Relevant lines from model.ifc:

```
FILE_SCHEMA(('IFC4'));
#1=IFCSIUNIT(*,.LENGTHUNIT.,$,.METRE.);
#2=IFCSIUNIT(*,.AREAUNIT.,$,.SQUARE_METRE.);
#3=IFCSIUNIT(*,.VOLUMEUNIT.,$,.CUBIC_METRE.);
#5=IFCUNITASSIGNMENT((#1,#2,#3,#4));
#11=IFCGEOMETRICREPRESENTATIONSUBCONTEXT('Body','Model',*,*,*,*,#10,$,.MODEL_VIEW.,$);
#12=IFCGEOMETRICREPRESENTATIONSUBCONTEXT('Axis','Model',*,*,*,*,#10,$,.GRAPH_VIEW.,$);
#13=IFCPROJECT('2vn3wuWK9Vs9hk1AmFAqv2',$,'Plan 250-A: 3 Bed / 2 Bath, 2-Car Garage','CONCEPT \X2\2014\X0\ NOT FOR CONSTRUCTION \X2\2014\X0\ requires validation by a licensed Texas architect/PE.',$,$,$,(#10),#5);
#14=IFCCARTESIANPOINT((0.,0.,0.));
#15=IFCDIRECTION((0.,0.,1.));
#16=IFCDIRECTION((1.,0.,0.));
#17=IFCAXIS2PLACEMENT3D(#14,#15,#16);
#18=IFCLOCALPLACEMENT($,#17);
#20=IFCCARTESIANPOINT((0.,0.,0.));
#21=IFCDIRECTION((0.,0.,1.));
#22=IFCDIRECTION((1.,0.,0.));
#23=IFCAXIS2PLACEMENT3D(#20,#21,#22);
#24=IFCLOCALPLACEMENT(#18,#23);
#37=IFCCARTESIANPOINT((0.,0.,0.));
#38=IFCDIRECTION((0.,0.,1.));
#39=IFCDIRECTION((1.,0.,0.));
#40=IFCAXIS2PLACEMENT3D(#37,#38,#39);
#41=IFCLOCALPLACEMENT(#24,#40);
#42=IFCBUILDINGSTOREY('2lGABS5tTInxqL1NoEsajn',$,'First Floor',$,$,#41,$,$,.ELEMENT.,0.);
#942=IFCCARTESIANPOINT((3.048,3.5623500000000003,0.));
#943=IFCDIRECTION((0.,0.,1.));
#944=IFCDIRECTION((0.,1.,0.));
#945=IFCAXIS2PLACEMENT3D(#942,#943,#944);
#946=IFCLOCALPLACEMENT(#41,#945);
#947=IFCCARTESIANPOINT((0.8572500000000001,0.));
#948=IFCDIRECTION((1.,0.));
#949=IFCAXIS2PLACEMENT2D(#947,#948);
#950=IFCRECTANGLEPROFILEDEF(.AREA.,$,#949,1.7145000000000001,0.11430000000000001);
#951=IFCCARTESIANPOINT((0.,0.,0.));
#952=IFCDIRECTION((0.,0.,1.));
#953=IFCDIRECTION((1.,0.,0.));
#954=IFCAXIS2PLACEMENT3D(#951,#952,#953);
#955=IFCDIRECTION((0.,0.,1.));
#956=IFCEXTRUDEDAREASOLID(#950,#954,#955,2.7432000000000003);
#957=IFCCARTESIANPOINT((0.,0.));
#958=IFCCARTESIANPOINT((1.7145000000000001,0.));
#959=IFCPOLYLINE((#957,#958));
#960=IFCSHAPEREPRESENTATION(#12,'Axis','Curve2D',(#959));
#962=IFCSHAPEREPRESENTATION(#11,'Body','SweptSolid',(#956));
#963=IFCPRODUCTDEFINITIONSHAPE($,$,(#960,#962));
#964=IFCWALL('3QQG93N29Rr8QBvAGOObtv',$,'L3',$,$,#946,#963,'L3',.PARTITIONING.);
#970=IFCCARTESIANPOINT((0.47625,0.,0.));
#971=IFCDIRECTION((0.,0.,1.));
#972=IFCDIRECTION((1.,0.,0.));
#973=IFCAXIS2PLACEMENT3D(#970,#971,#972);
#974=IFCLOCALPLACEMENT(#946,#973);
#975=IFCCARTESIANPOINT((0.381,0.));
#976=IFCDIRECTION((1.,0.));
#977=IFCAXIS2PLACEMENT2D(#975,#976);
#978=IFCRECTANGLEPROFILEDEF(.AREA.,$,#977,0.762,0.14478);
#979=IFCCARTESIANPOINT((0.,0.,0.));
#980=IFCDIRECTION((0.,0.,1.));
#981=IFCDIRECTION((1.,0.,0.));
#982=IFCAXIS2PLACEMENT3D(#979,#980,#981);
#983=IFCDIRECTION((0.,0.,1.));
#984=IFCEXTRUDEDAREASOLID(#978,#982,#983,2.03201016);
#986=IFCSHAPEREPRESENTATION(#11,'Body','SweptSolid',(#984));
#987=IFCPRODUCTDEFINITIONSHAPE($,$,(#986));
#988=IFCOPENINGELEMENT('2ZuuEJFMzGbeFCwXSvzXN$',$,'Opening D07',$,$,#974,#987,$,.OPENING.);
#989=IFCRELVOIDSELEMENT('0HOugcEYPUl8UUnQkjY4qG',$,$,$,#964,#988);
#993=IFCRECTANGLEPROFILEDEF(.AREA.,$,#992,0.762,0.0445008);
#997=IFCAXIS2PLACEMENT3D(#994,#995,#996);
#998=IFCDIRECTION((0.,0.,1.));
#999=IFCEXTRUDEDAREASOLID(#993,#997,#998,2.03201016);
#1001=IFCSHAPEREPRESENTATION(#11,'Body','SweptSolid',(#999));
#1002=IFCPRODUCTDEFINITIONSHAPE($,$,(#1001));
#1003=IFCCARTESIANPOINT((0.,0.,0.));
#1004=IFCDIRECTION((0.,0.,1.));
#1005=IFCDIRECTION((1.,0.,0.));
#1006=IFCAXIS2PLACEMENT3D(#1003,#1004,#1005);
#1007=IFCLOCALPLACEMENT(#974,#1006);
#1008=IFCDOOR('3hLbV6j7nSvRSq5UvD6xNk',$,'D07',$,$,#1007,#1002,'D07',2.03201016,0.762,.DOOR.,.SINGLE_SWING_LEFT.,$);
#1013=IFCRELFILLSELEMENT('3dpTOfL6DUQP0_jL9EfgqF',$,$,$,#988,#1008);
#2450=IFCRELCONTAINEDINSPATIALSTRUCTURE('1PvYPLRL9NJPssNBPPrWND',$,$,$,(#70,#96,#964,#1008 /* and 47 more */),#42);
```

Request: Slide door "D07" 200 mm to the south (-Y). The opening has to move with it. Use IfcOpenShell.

```python
import ifcopenshell
import ifcopenshell.api.geometry
import ifcopenshell.util.placement
import ifcopenshell.util.unit

model = ifcopenshell.open("model.ifc")
unit_scale = ifcopenshell.util.unit.calculate_unit_scale(model)

door = model.by_guid("3hLbV6j7nSvRSq5UvD6xNk")
opening = door.FillsVoids[0].RelatingOpeningElement
wall = opening.VoidsElements[0].RelatingBuildingElement

wall_matrix = ifcopenshell.util.placement.get_local_placement(wall.ObjectPlacement)
shift = wall_matrix[:3, 0] * -0.2 / unit_scale
before = ifcopenshell.util.placement.get_local_placement(door.ObjectPlacement)[:3, 3].copy()

# The door is placed relative to its opening, so it follows when the opening moves.
matrix = ifcopenshell.util.placement.get_local_placement(opening.ObjectPlacement)
matrix[:3, 3] += shift
ifcopenshell.api.geometry.edit_object_placement(
    model, product=opening, matrix=matrix, is_si=False, should_transform_children=True
)

after = ifcopenshell.util.placement.get_local_placement(door.ObjectPlacement)[:3, 3]
print("door moved by", (after - before).round(3) + 0.0)

model.write("model_rev.ifc")
```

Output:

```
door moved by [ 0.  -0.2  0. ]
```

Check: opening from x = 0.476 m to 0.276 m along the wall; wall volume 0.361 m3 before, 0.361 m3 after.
